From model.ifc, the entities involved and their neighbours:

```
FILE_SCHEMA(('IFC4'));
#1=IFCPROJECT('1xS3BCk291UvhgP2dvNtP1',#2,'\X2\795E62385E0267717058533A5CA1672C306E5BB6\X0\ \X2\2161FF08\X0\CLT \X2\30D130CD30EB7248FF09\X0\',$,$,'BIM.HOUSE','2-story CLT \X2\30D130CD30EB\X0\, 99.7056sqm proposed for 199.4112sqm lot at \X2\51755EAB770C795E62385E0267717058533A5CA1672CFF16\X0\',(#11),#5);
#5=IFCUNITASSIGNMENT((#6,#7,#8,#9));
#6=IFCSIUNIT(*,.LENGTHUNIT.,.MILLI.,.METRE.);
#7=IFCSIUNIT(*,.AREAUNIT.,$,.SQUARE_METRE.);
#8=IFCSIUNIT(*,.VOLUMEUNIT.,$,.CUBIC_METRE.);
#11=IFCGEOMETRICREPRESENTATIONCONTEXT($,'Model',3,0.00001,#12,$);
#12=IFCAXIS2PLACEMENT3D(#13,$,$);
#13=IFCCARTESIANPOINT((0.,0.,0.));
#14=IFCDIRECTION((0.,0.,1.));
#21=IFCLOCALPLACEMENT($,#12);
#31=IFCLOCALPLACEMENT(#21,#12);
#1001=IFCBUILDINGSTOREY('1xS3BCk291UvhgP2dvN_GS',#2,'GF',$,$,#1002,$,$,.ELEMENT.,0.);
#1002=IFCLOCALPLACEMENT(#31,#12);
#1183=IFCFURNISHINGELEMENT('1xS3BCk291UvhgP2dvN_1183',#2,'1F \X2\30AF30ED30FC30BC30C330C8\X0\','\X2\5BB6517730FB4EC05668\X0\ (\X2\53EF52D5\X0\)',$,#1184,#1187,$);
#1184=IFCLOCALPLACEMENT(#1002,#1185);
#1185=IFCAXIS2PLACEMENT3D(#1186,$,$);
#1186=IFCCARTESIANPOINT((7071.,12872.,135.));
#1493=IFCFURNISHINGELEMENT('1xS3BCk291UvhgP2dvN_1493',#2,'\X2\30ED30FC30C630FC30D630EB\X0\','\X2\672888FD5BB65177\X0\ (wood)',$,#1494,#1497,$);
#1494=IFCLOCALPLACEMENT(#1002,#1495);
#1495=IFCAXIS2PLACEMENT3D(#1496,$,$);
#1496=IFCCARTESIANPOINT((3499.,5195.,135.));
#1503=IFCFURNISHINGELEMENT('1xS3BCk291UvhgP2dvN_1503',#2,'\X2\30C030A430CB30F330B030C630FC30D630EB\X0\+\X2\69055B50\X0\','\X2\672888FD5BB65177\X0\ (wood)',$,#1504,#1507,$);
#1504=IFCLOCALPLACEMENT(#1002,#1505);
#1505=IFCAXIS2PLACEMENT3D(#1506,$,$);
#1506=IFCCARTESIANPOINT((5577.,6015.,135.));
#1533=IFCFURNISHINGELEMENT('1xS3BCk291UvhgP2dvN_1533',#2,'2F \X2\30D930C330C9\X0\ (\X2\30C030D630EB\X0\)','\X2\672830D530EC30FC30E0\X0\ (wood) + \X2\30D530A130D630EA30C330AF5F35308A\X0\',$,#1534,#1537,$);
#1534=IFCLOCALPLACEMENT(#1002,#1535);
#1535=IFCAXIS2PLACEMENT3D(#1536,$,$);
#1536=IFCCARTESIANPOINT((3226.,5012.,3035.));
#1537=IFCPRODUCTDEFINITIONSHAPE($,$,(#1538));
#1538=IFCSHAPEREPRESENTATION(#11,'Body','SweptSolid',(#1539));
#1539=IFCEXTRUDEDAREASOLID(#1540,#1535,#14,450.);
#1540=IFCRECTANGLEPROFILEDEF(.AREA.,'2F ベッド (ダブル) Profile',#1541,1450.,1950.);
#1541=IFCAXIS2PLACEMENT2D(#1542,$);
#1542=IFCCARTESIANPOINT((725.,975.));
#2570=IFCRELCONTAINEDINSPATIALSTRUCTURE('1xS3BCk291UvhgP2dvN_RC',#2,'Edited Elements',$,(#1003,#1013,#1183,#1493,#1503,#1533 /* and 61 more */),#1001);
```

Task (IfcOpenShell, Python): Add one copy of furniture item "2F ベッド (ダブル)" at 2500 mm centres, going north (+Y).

```python
import numpy as np
import ifcopenshell
import ifcopenshell.api.geometry
import ifcopenshell.api.root
import ifcopenshell.util.element
import ifcopenshell.util.placement
import ifcopenshell.util.unit

model = ifcopenshell.open("model.ifc")
unit_scale = ifcopenshell.util.unit.calculate_unit_scale(model)


def reuse_history(source, copy):
    """copy_class also copies each property set's owner history, people and application; keep the originals."""
    for rel in copy.IsDefinedBy:
        if rel.is_a("IfcRelDefinesByProperties") and (history := rel.RelatingPropertyDefinition.OwnerHistory):
            rel.RelatingPropertyDefinition.OwnerHistory = source.OwnerHistory
            ifcopenshell.util.element.remove_deep2(model, history)


source = model.by_guid("1xS3BCk291UvhgP2dvN_1533")
base = ifcopenshell.util.placement.get_local_placement(source.ObjectPlacement)
step = np.array([0.0, 1.0, 0.0]) * 2.5 / unit_scale

for i in range(1, 2):
    copy = ifcopenshell.api.root.copy_class(model, product=source)
    copy.Representation = ifcopenshell.util.element.copy_deep(
        model, source.Representation, exclude=["IfcGeometricRepresentationContext", "IfcRepresentationMap"]
    )
    reuse_history(source, copy)
    matrix = base.copy()
    matrix[:3, 3] += i * step
    print("added at", matrix[:3, 3].round(3) + 0.0)
    ifcopenshell.api.geometry.edit_object_placement(model, product=copy, matrix=matrix, is_si=False)

model.write("model_edited.ifc")
```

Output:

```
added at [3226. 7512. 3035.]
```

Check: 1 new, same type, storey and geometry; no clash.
